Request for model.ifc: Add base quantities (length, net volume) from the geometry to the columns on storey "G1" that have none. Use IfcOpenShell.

First a look at what the model holds.

```python
import ifcopenshell
import ifcopenshell.util.element
import ifcopenshell.util.unit

model = ifcopenshell.open("model.ifc")
print(model.schema)
for unit_type in ("LENGTHUNIT", "AREAUNIT", "VOLUMEUNIT"):
    print(unit_type, ifcopenshell.util.unit.calculate_unit_scale(model, unit_type))
storey = next(s for s in model.by_type("IfcBuildingStorey") if s.Name == "G1")
columns = [e for e in ifcopenshell.util.element.get_decomposition(storey) if e.is_a("IfcColumn")]
for e in sorted(columns, key=lambda e: e.id()):
    print(e.id(), e.is_a(), e.Name, list(ifcopenshell.util.element.get_psets(e, qtos_only=True)), sep=" | ")
```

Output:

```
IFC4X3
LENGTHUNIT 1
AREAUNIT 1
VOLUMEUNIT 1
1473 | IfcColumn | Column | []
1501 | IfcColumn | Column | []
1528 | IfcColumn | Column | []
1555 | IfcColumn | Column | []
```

```python
import ifcopenshell
import ifcopenshell.api.pset
import ifcopenshell.geom
import ifcopenshell.util.element
import ifcopenshell.util.shape
import ifcopenshell.util.unit

model = ifcopenshell.open("model.ifc")
unit_scale = ifcopenshell.util.unit.calculate_unit_scale(model)
volume_scale = ifcopenshell.util.unit.calculate_unit_scale(model, "VOLUMEUNIT")
settings = ifcopenshell.geom.settings()

storey = next(s for s in model.by_type("IfcBuildingStorey") if s.Name == "G1")
columns = [e for e in ifcopenshell.util.element.get_decomposition(storey) if e.is_a("IfcColumn")]

for e in sorted(columns, key=lambda e: e.id()):
    if ifcopenshell.util.element.get_psets(e, qtos_only=True, should_inherit=False):
        continue
    # Geometry comes back in metres, in the element's own axes.
    shape = ifcopenshell.geom.create_shape(settings, e)
    values = {
        "Length": ifcopenshell.util.shape.get_z(shape.geometry) / unit_scale,
        "NetVolume": ifcopenshell.util.shape.get_volume(shape.geometry) / volume_scale,
    }
    qto = ifcopenshell.api.pset.add_qto(model, product=e, name="Qto_ColumnBaseQuantities")
    ifcopenshell.api.pset.edit_qto(model, qto=qto, properties=values)
    print(e.id(), {k: round(v, 3) for k, v in values.items()})

model.write("model-out.ifc")
```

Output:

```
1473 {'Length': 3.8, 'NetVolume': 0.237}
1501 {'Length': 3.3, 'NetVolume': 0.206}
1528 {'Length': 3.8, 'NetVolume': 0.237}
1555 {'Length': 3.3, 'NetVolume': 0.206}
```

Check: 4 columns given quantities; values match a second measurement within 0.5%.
